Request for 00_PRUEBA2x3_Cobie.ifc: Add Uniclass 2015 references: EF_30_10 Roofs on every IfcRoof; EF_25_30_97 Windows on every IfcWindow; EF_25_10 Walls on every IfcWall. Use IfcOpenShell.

First a look at what the model holds.

```python
import ifcopenshell

model = ifcopenshell.open("00_PRUEBA2x3_Cobie.ifc")
print(model.schema)
print("classifications:", [c.Name for c in model.by_type("IfcClassification")])
for ifc_class in ("IfcDoor", "IfcRoof", "IfcStair", "IfcWall", "IfcWindow"):
    print(ifc_class, len(model.by_type(ifc_class)))
```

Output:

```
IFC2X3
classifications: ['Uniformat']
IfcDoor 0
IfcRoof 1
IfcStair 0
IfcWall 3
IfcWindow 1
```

```python
import ifcopenshell
import ifcopenshell.api.classification

model = ifcopenshell.open("00_PRUEBA2x3_Cobie.ifc")

# IFC2X3 requires Source and Edition and has no link from the project to the system.
system = model.create_entity("IfcClassification", Source="NBS", Edition="2015", Name="Uniclass 2015")

codes = {
    "IfcRoof": ("EF_30_10", "Roofs"),
    "IfcWindow": ("EF_25_30_97", "Windows"),
    "IfcWall": ("EF_25_10", "Walls"),
}
for ifc_class, (code, name) in codes.items():
    products = model.by_type(ifc_class)
    ifcopenshell.api.classification.add_reference(
        model, products=products, classification=system, identification=code, name=name
    )
    print(code, len(products))

model.write("00_PRUEBA2x3_Cobie_rev.ifc")
```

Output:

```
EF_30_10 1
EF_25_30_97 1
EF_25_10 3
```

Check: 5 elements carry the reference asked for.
